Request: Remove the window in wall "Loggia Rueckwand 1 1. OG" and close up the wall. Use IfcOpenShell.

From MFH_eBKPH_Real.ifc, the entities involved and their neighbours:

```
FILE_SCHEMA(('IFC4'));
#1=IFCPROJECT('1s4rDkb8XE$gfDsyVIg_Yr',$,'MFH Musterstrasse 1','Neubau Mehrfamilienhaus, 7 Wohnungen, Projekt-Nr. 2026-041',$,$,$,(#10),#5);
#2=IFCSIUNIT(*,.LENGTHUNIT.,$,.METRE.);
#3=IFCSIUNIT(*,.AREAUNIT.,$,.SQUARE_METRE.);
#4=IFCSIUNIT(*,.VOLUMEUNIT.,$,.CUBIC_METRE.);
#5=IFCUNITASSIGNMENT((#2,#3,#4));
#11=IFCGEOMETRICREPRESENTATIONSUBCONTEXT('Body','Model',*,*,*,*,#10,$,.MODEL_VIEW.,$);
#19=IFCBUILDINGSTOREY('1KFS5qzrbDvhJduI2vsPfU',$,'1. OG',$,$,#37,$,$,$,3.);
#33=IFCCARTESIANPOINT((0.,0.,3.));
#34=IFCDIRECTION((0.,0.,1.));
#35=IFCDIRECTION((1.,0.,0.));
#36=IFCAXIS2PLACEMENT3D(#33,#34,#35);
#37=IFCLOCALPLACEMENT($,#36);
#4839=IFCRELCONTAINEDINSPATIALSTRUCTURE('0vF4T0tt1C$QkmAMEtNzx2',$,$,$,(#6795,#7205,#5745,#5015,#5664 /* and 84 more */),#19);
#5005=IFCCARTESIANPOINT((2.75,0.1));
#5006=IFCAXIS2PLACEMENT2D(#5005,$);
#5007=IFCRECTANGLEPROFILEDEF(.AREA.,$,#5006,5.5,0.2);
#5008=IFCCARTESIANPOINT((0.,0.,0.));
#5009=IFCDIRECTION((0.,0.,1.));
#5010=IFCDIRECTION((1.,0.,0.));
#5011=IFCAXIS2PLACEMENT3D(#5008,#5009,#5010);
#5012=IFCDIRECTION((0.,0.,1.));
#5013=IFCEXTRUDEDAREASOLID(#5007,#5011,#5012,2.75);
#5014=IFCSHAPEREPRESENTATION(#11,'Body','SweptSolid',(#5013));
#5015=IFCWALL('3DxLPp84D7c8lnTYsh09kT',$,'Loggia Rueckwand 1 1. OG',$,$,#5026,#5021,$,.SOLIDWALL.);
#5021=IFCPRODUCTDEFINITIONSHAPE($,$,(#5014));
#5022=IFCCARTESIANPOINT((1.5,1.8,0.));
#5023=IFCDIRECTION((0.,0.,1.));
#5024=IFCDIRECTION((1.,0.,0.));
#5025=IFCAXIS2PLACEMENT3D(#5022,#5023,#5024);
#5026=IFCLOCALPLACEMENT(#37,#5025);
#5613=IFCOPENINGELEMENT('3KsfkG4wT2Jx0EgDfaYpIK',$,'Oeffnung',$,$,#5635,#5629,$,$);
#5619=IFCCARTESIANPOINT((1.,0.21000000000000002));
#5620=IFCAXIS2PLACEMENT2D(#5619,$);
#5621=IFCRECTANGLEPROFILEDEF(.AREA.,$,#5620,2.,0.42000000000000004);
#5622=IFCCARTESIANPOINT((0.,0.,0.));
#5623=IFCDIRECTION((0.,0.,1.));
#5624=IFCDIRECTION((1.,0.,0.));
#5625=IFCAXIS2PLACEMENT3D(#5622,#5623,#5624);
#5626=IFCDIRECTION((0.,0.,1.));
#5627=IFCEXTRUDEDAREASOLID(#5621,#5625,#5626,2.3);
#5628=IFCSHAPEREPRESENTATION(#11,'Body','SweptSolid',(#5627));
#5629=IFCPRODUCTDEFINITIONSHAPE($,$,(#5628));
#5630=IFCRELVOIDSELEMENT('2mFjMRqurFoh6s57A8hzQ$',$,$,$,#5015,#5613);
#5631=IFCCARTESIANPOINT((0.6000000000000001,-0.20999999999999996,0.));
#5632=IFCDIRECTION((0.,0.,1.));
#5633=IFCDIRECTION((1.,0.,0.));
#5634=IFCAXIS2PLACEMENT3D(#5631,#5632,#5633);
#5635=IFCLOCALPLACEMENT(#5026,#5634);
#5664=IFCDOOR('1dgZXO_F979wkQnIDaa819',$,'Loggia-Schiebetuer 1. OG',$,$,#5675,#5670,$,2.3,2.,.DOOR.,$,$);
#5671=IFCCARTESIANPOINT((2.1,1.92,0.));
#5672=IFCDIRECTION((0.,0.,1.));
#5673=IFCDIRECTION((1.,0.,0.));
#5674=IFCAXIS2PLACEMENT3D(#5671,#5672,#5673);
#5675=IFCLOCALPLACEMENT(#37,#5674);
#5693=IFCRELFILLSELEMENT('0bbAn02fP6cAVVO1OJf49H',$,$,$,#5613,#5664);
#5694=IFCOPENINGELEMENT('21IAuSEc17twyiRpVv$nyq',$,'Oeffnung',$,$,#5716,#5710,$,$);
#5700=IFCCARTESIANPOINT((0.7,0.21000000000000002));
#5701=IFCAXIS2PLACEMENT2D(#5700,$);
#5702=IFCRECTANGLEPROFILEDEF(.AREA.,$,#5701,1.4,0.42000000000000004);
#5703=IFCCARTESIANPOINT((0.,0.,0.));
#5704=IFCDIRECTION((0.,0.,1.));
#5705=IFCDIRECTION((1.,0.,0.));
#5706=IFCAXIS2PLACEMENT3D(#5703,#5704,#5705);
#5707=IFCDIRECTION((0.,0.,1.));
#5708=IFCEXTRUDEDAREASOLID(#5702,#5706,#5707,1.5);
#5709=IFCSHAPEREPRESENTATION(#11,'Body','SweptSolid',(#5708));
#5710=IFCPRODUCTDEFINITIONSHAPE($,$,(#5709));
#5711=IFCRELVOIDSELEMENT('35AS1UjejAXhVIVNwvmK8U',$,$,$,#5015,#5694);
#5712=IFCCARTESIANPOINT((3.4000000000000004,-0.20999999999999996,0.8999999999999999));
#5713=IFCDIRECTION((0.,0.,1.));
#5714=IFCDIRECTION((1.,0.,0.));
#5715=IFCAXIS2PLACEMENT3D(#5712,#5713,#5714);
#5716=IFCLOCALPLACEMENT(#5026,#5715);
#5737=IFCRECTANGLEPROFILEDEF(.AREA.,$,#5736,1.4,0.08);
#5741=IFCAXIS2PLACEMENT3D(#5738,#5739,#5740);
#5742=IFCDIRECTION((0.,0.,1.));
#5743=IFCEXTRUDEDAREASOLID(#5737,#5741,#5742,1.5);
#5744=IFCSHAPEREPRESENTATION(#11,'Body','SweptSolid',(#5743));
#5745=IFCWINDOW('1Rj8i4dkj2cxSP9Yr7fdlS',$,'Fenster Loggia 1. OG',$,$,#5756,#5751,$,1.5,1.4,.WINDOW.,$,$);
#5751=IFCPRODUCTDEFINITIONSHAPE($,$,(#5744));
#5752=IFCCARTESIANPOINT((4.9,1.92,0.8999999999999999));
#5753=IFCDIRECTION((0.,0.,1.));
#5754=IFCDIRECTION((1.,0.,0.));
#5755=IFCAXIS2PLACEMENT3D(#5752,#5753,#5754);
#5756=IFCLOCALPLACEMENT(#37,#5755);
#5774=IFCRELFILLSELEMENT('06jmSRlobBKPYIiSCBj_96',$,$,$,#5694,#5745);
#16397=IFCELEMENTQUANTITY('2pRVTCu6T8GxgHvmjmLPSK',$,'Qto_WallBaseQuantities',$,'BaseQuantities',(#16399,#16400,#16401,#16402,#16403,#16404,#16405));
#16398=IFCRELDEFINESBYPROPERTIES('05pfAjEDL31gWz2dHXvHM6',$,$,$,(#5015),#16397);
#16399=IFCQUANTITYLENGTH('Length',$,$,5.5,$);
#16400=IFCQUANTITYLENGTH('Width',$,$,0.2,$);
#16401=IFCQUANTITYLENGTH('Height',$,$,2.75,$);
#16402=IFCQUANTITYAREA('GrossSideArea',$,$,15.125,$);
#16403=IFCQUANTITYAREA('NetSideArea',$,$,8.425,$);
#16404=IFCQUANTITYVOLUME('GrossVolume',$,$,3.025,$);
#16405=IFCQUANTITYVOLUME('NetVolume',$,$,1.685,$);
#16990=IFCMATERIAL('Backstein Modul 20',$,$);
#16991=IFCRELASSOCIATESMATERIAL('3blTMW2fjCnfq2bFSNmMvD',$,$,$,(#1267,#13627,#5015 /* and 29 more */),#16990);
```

```python
import ifcopenshell
import ifcopenshell.api.feature
import ifcopenshell.api.pset
import ifcopenshell.api.root
import ifcopenshell.geom
import ifcopenshell.util.element
import ifcopenshell.util.shape
import ifcopenshell.util.unit

model = ifcopenshell.open("MFH_eBKPH_Real.ifc")
area_scale = ifcopenshell.util.unit.calculate_unit_scale(model, "AREAUNIT")
volume_scale = ifcopenshell.util.unit.calculate_unit_scale(model, "VOLUMEUNIT")
settings = ifcopenshell.geom.settings()


def volume(element):
    """Net volume in cubic metres, openings subtracted."""
    shape = ifcopenshell.geom.create_shape(settings, element)
    return ifcopenshell.util.shape.get_volume(shape.geometry)


window = model.by_id(5745)
opening = window.FillsVoids[0].RelatingOpeningElement
wall = opening.VoidsElements[0].RelatingBuildingElement
before = volume(wall)

ifcopenshell.api.root.remove_product(model, product=window)
ifcopenshell.api.feature.remove_feature(model, feature=opening)

after = volume(wall)
thickness = 0.2  # wall thickness in metres

# Update the wall's stored quantities.
qto = model.by_id(ifcopenshell.util.element.get_pset(wall, "Qto_WallBaseQuantities", should_inherit=False)["id"])
ifcopenshell.api.pset.edit_qto(model, qto=qto, properties={
    "NetSideArea": after / thickness / area_scale,
    "NetVolume": after / volume_scale,
})

print(f"wall volume {before:.3f} -> {after:.3f} m3")

model.write("MFH_eBKPH_Real_updated.ifc")
```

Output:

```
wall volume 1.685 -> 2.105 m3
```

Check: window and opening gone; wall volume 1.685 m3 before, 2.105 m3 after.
